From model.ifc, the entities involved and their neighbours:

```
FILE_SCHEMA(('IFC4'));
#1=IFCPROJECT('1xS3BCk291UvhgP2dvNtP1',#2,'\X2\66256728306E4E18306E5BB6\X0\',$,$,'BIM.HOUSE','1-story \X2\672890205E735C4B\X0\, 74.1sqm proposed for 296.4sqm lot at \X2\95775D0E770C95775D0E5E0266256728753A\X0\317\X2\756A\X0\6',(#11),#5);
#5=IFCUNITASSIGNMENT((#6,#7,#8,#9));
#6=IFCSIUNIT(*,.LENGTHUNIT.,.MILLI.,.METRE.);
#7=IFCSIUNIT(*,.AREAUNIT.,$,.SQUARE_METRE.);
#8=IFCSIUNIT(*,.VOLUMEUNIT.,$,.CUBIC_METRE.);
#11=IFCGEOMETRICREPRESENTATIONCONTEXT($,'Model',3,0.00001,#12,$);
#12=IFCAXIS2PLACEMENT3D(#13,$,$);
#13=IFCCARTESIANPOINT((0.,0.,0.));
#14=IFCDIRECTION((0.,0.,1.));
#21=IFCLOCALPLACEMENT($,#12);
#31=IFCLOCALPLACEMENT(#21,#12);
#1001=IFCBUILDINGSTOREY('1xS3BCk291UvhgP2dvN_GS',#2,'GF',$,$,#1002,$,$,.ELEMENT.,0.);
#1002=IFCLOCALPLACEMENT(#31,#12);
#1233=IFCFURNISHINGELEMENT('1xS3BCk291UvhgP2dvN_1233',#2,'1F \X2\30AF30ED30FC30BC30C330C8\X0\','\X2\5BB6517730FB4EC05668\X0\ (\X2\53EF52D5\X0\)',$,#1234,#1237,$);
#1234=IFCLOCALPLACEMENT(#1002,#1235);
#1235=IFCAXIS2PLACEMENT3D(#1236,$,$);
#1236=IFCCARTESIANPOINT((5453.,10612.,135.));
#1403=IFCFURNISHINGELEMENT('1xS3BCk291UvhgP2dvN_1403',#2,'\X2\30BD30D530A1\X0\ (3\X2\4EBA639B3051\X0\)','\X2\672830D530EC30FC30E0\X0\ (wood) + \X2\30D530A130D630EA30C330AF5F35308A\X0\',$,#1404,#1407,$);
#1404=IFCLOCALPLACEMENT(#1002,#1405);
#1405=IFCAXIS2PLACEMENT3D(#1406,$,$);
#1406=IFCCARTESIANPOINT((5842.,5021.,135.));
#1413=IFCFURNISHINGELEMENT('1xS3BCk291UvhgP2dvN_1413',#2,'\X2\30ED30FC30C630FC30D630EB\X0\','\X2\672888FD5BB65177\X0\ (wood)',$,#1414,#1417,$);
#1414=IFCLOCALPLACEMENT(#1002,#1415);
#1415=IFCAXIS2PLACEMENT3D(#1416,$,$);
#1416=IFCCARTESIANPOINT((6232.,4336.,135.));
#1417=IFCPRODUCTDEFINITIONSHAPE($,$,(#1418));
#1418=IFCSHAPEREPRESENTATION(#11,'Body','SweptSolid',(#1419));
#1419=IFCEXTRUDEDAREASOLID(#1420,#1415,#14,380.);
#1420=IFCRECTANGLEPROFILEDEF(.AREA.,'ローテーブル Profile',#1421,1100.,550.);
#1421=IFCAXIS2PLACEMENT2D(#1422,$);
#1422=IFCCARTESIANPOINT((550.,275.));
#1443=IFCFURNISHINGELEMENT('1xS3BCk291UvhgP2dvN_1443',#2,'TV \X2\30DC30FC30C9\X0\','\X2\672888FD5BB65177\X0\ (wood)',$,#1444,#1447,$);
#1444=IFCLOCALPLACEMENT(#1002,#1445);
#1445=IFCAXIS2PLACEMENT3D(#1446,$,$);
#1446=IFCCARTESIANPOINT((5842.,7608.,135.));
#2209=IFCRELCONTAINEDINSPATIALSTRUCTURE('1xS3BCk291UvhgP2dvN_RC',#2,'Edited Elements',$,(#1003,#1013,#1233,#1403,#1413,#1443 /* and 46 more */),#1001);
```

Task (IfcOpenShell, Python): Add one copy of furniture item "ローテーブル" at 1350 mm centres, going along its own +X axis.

```python
import ifcopenshell
import ifcopenshell.api.geometry
import ifcopenshell.api.root
import ifcopenshell.util.element
import ifcopenshell.util.placement
import ifcopenshell.util.unit

model = ifcopenshell.open("model.ifc")
unit_scale = ifcopenshell.util.unit.calculate_unit_scale(model)


def reuse_history(source, copy):
    """copy_class also copies each property set's owner history, people and application; keep the originals."""
    for rel in copy.IsDefinedBy:
        if rel.is_a("IfcRelDefinesByProperties") and (history := rel.RelatingPropertyDefinition.OwnerHistory):
            rel.RelatingPropertyDefinition.OwnerHistory = source.OwnerHistory
            ifcopenshell.util.element.remove_deep2(model, history)


source = model.by_id(1413)
base = ifcopenshell.util.placement.get_local_placement(source.ObjectPlacement)
step = base[:3, 0] * 1.35 / unit_scale

for i in range(1, 2):
    copy = ifcopenshell.api.root.copy_class(model, product=source)
    copy.Representation = ifcopenshell.util.element.copy_deep(
        model, source.Representation, exclude=["IfcGeometricRepresentationContext", "IfcRepresentationMap"]
    )
    reuse_history(source, copy)
    matrix = base.copy()
    matrix[:3, 3] += i * step
    print("added at", matrix[:3, 3].round(3) + 0.0)
    ifcopenshell.api.geometry.edit_object_placement(model, product=copy, matrix=matrix, is_si=False)

model.write("model-out.ifc")
```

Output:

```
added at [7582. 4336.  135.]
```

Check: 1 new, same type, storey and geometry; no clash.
